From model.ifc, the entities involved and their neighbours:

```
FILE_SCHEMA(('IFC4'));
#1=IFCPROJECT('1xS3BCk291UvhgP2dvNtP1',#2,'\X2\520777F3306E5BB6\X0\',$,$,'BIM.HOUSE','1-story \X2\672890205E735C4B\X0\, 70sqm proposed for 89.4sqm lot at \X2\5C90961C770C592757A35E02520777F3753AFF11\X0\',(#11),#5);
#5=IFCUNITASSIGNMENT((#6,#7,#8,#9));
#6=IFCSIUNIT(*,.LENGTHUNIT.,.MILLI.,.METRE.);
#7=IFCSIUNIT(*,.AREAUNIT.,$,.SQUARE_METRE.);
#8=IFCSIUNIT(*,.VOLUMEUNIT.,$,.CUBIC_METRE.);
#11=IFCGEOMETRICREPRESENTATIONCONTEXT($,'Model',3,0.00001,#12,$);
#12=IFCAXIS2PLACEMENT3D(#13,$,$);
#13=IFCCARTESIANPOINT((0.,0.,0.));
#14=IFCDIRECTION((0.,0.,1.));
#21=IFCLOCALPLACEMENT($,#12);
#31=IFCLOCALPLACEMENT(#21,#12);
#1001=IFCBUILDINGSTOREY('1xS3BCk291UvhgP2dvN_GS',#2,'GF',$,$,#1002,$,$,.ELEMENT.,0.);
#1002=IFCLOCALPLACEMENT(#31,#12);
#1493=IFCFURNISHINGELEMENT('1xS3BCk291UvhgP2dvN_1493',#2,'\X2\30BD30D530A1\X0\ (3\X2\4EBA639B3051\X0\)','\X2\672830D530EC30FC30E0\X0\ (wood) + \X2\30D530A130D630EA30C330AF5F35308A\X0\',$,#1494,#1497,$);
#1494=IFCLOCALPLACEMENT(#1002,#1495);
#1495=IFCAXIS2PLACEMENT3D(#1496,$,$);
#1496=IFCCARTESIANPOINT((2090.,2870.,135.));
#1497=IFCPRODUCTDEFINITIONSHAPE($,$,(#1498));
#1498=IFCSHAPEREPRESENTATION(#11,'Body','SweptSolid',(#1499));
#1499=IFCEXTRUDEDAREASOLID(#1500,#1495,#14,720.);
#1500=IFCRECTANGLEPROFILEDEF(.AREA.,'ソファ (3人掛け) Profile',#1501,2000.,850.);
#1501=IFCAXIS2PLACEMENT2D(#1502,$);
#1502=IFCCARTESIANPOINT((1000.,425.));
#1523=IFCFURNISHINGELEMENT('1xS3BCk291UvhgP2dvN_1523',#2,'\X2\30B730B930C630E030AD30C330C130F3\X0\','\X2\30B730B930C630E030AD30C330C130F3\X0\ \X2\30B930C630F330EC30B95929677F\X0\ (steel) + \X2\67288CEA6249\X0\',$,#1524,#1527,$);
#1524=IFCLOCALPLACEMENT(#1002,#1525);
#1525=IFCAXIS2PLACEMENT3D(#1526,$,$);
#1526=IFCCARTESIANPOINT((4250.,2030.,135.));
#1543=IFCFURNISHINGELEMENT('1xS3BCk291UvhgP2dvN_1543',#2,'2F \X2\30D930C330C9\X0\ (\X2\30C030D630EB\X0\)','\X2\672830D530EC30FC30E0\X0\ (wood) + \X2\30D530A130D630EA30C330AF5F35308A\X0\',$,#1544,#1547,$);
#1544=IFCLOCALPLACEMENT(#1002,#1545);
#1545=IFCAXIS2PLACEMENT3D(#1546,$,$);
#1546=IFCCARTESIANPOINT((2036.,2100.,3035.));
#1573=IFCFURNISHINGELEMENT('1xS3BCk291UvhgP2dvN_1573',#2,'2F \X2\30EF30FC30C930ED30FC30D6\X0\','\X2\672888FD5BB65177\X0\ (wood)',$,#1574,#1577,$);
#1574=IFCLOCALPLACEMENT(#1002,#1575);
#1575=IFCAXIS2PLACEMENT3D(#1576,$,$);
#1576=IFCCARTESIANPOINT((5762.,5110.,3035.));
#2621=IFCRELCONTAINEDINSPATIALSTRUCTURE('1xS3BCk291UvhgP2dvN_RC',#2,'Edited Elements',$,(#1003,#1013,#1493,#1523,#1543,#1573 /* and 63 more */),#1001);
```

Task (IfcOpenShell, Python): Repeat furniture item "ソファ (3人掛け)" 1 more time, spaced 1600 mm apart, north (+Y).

```python
import numpy as np
import ifcopenshell
import ifcopenshell.api.geometry
import ifcopenshell.api.root
import ifcopenshell.util.element
import ifcopenshell.util.placement
import ifcopenshell.util.unit

model = ifcopenshell.open("model.ifc")
unit_scale = ifcopenshell.util.unit.calculate_unit_scale(model)


def reuse_history(source, copy):
    """copy_class also copies each property set's owner history, people and application; keep the originals."""
    for rel in copy.IsDefinedBy:
        if rel.is_a("IfcRelDefinesByProperties") and (history := rel.RelatingPropertyDefinition.OwnerHistory):
            rel.RelatingPropertyDefinition.OwnerHistory = source.OwnerHistory
            ifcopenshell.util.element.remove_deep2(model, history)


source = model.by_guid("1xS3BCk291UvhgP2dvN_1493")
base = ifcopenshell.util.placement.get_local_placement(source.ObjectPlacement)
step = np.array([0.0, 1.0, 0.0]) * 1.6 / unit_scale

for i in range(1, 2):
    copy = ifcopenshell.api.root.copy_class(model, product=source)
    copy.Representation = ifcopenshell.util.element.copy_deep(
        model, source.Representation, exclude=["IfcGeometricRepresentationContext", "IfcRepresentationMap"]
    )
    reuse_history(source, copy)
    matrix = base.copy()
    matrix[:3, 3] += i * step
    print("added at", matrix[:3, 3].round(3) + 0.0)
    ifcopenshell.api.geometry.edit_object_placement(model, product=copy, matrix=matrix, is_si=False)

model.write("model_v2.ifc")
```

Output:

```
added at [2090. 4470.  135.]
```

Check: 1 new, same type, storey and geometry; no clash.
